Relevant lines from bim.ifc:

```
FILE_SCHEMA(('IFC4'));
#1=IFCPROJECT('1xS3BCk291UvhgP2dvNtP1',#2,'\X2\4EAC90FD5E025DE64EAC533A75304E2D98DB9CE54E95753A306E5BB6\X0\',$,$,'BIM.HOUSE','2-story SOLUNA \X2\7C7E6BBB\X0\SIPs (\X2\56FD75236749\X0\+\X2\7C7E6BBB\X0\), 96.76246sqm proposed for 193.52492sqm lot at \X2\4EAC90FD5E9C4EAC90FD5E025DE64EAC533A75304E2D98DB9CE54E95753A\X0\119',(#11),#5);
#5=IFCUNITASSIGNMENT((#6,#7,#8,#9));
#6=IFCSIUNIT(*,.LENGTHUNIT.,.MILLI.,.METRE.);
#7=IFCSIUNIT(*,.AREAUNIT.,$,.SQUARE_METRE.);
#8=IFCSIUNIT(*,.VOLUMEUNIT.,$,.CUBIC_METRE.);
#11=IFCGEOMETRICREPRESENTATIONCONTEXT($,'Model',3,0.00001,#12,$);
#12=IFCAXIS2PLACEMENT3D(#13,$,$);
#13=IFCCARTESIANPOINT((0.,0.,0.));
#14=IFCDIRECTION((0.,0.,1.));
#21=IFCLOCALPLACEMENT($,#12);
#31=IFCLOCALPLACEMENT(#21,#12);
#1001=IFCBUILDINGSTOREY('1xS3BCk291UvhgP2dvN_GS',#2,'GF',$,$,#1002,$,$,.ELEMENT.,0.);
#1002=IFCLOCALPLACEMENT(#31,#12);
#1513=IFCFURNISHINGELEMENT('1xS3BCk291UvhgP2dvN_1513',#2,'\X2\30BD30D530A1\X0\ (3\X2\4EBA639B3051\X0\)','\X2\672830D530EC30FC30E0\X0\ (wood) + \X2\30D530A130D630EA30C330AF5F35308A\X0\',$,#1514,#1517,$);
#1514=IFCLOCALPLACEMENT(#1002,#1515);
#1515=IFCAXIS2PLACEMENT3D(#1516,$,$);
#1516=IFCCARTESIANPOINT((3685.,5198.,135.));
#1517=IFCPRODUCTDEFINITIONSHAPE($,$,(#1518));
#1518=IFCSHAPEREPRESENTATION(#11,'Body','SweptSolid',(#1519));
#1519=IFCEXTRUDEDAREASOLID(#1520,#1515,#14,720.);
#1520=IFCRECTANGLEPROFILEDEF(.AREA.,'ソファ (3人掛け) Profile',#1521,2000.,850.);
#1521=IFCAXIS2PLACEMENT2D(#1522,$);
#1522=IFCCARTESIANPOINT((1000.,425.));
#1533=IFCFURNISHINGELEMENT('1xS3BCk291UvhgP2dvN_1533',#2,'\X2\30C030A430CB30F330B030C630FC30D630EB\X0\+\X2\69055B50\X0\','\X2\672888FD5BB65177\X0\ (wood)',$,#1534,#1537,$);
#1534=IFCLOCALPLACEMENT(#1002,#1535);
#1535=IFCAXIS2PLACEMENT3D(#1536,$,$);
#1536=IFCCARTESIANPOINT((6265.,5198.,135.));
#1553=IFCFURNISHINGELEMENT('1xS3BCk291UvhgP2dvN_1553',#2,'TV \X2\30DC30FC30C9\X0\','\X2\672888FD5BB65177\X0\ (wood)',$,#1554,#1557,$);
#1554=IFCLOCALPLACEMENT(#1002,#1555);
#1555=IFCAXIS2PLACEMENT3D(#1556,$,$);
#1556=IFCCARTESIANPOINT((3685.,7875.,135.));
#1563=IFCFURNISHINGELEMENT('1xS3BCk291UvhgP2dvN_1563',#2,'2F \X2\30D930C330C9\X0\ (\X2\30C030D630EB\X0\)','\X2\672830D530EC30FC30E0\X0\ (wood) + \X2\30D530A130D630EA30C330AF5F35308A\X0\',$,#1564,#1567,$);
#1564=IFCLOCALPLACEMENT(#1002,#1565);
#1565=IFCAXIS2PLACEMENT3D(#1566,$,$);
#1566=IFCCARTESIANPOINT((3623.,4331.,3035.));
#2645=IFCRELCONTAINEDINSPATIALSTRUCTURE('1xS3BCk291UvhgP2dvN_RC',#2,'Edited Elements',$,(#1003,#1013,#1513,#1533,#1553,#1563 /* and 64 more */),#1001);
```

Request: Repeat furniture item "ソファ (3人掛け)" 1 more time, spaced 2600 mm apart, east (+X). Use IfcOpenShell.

```python
import numpy as np
import ifcopenshell
import ifcopenshell.api.geometry
import ifcopenshell.api.root
import ifcopenshell.util.element
import ifcopenshell.util.placement
import ifcopenshell.util.unit

model = ifcopenshell.open("bim.ifc")
unit_scale = ifcopenshell.util.unit.calculate_unit_scale(model)


def reuse_history(source, copy):
    """copy_class also copies each property set's owner history, people and application; keep the originals."""
    for rel in copy.IsDefinedBy:
        if rel.is_a("IfcRelDefinesByProperties") and (history := rel.RelatingPropertyDefinition.OwnerHistory):
            rel.RelatingPropertyDefinition.OwnerHistory = source.OwnerHistory
            ifcopenshell.util.element.remove_deep2(model, history)


source = model.by_id(1513)
base = ifcopenshell.util.placement.get_local_placement(source.ObjectPlacement)
step = np.array([1.0, 0.0, 0.0]) * 2.6 / unit_scale

for i in range(1, 2):
    copy = ifcopenshell.api.root.copy_class(model, product=source)
    copy.Representation = ifcopenshell.util.element.copy_deep(
        model, source.Representation, exclude=["IfcGeometricRepresentationContext", "IfcRepresentationMap"]
    )
    reuse_history(source, copy)
    matrix = base.copy()
    matrix[:3, 3] += i * step
    print("added at", matrix[:3, 3].round(3) + 0.0)
    ifcopenshell.api.geometry.edit_object_placement(model, product=copy, matrix=matrix, is_si=False)

model.write("bim_v2.ifc")
```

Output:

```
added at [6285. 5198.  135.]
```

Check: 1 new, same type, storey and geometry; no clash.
